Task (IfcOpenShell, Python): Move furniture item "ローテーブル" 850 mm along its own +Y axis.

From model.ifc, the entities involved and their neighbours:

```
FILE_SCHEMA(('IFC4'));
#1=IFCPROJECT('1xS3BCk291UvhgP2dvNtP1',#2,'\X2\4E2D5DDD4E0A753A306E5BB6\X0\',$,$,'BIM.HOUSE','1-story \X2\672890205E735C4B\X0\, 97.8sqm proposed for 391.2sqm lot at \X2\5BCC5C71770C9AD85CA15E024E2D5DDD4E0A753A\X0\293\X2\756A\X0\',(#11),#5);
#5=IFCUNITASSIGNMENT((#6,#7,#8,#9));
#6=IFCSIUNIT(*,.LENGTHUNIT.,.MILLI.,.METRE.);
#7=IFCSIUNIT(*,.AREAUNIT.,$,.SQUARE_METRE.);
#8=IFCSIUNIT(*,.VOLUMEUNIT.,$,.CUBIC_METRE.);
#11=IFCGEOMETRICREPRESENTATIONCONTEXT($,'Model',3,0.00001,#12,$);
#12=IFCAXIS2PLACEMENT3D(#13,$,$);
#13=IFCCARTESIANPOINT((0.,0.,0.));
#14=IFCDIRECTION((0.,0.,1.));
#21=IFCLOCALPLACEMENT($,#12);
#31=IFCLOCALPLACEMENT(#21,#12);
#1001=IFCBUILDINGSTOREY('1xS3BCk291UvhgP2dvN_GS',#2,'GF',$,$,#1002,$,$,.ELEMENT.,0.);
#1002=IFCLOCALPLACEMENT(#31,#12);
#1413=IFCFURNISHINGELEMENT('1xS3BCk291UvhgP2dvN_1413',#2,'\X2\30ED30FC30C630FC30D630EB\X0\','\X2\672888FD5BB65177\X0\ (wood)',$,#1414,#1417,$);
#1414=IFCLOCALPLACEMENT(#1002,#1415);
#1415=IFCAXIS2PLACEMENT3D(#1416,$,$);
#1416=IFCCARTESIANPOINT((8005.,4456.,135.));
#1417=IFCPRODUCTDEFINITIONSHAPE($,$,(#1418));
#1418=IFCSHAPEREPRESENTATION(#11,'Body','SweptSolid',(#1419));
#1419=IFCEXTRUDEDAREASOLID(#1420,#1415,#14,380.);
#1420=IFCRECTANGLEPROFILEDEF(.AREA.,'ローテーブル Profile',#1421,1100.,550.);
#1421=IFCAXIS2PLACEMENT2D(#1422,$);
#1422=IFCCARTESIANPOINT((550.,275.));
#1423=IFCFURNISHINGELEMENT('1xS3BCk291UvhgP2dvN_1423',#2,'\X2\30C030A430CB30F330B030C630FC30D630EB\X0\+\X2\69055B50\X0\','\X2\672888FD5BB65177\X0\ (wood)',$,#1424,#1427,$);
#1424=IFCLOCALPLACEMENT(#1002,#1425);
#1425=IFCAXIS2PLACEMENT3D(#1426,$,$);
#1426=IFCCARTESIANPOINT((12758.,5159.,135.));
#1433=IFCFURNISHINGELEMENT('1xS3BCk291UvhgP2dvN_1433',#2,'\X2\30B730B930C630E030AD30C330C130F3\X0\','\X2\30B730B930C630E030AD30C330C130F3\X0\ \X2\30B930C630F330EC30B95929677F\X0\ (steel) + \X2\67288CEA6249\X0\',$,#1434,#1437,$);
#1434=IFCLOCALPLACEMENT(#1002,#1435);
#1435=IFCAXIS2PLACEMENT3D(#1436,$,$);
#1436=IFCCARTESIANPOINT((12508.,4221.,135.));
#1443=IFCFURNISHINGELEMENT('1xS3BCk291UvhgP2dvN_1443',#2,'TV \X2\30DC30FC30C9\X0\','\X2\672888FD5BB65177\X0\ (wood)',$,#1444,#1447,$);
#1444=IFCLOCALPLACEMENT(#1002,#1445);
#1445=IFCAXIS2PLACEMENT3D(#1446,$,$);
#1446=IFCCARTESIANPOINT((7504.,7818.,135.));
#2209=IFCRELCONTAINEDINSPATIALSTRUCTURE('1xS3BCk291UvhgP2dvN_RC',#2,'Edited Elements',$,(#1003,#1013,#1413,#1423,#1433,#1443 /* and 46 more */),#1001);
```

```python
import ifcopenshell
import ifcopenshell.api.geometry
import ifcopenshell.util.placement

model = ifcopenshell.open("model.ifc")

item = model.by_guid("1xS3BCk291UvhgP2dvN_1413")
matrix = ifcopenshell.util.placement.get_local_placement(item.ObjectPlacement)
matrix[:3, 3] += matrix[:3, 1] * 850.0
ifcopenshell.api.geometry.edit_object_placement(model, product=item, matrix=matrix, is_si=False)

print(ifcopenshell.util.placement.get_local_placement(item.ObjectPlacement).round(3) + 0.0)

model.write("model-out.ifc")
```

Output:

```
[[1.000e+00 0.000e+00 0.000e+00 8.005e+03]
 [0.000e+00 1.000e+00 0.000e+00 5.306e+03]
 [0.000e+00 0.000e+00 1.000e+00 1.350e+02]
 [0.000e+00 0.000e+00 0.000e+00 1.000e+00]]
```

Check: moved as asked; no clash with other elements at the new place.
